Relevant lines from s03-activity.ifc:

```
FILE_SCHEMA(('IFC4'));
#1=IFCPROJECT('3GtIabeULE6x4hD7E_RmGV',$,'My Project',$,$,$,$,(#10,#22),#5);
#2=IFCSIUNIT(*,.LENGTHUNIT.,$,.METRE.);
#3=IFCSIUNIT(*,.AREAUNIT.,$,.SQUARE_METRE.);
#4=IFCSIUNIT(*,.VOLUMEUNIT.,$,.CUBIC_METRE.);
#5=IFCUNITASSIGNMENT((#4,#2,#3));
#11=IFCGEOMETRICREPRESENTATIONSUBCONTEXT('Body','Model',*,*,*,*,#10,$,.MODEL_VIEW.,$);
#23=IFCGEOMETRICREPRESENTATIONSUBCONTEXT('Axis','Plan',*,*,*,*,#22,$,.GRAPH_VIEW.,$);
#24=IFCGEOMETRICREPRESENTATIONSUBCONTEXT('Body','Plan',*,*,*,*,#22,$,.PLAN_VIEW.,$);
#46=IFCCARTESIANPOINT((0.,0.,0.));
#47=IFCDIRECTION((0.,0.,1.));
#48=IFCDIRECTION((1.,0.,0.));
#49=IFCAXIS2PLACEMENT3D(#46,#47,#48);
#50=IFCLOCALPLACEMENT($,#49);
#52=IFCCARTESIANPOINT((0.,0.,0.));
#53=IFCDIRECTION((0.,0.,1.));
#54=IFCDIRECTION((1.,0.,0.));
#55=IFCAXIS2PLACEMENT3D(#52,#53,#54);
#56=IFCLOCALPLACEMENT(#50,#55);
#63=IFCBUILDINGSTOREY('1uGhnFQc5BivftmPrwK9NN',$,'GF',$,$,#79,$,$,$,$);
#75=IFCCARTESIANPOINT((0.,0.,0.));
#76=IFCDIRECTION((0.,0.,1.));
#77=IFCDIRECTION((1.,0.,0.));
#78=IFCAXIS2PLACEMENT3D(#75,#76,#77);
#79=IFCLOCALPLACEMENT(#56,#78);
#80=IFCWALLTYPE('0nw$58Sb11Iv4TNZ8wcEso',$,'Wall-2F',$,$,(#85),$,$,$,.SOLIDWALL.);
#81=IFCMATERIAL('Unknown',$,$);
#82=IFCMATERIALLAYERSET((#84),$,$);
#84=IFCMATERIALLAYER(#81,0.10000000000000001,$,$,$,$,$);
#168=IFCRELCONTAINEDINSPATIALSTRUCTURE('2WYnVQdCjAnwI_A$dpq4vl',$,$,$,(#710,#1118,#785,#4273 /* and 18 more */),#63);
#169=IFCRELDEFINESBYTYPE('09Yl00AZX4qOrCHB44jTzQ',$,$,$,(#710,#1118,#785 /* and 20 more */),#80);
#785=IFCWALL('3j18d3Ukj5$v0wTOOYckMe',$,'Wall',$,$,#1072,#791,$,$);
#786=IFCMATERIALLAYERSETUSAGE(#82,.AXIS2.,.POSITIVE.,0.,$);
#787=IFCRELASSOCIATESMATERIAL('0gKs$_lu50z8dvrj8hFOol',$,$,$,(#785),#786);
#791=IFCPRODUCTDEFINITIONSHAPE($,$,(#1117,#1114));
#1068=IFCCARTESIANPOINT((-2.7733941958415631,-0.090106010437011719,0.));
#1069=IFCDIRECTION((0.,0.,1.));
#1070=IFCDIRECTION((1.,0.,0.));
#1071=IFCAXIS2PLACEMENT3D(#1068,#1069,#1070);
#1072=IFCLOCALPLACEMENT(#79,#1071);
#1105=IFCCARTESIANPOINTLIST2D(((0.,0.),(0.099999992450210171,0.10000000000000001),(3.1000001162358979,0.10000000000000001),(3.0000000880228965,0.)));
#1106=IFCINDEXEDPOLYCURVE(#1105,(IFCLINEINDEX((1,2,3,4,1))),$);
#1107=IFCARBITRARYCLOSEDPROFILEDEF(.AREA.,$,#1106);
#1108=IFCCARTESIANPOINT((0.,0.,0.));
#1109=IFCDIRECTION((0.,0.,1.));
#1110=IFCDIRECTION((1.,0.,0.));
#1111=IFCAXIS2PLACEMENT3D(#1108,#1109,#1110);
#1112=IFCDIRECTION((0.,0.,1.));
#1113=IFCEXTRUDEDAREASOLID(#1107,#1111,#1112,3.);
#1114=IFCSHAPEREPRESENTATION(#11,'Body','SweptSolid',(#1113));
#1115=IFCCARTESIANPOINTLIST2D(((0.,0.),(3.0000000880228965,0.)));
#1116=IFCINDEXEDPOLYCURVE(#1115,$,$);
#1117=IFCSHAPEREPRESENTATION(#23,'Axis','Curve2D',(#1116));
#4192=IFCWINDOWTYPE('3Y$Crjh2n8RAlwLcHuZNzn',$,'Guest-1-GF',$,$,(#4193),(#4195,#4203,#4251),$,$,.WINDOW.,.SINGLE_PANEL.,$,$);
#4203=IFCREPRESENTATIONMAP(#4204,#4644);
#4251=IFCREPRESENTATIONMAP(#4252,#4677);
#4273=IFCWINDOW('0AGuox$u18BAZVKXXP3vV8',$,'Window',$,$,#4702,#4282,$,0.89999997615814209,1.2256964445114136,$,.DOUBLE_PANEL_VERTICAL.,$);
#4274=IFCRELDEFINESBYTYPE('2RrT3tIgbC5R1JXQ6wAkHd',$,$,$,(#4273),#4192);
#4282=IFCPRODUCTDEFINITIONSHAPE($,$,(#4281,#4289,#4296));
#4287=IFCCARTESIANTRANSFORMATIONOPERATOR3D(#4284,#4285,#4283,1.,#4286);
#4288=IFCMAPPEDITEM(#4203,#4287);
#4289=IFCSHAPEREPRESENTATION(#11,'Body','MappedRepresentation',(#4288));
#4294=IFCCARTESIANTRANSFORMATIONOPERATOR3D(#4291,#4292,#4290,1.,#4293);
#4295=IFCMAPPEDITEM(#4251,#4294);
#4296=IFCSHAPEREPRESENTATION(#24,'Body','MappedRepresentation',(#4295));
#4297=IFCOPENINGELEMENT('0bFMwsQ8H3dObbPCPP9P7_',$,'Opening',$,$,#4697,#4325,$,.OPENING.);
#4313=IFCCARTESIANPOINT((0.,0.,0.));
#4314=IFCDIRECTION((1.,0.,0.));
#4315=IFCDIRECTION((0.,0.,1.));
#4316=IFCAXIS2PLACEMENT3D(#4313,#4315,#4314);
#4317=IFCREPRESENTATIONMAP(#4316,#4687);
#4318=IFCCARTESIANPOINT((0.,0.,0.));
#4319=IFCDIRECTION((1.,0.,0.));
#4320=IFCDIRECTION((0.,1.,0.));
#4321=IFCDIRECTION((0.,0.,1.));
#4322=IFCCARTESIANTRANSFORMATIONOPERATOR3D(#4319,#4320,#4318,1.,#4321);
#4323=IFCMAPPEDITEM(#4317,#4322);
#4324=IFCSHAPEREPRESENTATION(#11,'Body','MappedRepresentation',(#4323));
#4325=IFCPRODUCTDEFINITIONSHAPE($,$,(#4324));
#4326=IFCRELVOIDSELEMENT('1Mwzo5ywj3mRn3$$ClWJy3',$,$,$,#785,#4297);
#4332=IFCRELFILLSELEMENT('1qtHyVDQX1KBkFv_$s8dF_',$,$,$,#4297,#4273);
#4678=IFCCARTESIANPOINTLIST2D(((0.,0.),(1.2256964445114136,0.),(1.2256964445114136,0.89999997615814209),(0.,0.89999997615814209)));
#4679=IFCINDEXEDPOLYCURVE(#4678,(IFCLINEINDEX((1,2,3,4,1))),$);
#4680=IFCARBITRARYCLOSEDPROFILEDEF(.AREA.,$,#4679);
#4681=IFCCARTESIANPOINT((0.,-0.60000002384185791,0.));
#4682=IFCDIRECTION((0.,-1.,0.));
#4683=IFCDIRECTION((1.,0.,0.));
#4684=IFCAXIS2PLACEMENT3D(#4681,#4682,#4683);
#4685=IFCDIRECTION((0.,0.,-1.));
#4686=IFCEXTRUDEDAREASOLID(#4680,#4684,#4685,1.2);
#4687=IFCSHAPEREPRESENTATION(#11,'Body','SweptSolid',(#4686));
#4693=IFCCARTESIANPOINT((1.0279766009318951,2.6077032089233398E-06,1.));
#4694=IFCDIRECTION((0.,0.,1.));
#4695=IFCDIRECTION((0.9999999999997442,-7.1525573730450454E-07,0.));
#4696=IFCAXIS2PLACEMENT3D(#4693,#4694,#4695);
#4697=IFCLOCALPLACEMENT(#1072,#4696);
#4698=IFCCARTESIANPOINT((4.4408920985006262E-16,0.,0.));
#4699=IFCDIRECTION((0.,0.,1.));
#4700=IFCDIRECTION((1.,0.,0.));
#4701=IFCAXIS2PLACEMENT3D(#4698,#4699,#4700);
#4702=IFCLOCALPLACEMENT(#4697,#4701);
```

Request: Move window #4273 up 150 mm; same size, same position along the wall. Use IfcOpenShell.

```python
import numpy as np
import ifcopenshell
import ifcopenshell.api.geometry
import ifcopenshell.util.placement
import ifcopenshell.util.unit

model = ifcopenshell.open("s03-activity.ifc")
unit_scale = ifcopenshell.util.unit.calculate_unit_scale(model)

window = model.by_guid("0AGuox$u18BAZVKXXP3vV8")
opening = window.FillsVoids[0].RelatingOpeningElement
dz = 0.15 / unit_scale

shift = np.array([0.0, 0.0, dz])
# The window is placed relative to its opening, so it follows when the opening moves.
matrix = ifcopenshell.util.placement.get_local_placement(opening.ObjectPlacement)
matrix[:3, 3] += shift
ifcopenshell.api.geometry.edit_object_placement(
    model, product=opening, matrix=matrix, is_si=False, should_transform_children=True
)

print(f"moved by {dz * unit_scale:+.3f} m")

model.write("s03-activity_v2.ifc")
```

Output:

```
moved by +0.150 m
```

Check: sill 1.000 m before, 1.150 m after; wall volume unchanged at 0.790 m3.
